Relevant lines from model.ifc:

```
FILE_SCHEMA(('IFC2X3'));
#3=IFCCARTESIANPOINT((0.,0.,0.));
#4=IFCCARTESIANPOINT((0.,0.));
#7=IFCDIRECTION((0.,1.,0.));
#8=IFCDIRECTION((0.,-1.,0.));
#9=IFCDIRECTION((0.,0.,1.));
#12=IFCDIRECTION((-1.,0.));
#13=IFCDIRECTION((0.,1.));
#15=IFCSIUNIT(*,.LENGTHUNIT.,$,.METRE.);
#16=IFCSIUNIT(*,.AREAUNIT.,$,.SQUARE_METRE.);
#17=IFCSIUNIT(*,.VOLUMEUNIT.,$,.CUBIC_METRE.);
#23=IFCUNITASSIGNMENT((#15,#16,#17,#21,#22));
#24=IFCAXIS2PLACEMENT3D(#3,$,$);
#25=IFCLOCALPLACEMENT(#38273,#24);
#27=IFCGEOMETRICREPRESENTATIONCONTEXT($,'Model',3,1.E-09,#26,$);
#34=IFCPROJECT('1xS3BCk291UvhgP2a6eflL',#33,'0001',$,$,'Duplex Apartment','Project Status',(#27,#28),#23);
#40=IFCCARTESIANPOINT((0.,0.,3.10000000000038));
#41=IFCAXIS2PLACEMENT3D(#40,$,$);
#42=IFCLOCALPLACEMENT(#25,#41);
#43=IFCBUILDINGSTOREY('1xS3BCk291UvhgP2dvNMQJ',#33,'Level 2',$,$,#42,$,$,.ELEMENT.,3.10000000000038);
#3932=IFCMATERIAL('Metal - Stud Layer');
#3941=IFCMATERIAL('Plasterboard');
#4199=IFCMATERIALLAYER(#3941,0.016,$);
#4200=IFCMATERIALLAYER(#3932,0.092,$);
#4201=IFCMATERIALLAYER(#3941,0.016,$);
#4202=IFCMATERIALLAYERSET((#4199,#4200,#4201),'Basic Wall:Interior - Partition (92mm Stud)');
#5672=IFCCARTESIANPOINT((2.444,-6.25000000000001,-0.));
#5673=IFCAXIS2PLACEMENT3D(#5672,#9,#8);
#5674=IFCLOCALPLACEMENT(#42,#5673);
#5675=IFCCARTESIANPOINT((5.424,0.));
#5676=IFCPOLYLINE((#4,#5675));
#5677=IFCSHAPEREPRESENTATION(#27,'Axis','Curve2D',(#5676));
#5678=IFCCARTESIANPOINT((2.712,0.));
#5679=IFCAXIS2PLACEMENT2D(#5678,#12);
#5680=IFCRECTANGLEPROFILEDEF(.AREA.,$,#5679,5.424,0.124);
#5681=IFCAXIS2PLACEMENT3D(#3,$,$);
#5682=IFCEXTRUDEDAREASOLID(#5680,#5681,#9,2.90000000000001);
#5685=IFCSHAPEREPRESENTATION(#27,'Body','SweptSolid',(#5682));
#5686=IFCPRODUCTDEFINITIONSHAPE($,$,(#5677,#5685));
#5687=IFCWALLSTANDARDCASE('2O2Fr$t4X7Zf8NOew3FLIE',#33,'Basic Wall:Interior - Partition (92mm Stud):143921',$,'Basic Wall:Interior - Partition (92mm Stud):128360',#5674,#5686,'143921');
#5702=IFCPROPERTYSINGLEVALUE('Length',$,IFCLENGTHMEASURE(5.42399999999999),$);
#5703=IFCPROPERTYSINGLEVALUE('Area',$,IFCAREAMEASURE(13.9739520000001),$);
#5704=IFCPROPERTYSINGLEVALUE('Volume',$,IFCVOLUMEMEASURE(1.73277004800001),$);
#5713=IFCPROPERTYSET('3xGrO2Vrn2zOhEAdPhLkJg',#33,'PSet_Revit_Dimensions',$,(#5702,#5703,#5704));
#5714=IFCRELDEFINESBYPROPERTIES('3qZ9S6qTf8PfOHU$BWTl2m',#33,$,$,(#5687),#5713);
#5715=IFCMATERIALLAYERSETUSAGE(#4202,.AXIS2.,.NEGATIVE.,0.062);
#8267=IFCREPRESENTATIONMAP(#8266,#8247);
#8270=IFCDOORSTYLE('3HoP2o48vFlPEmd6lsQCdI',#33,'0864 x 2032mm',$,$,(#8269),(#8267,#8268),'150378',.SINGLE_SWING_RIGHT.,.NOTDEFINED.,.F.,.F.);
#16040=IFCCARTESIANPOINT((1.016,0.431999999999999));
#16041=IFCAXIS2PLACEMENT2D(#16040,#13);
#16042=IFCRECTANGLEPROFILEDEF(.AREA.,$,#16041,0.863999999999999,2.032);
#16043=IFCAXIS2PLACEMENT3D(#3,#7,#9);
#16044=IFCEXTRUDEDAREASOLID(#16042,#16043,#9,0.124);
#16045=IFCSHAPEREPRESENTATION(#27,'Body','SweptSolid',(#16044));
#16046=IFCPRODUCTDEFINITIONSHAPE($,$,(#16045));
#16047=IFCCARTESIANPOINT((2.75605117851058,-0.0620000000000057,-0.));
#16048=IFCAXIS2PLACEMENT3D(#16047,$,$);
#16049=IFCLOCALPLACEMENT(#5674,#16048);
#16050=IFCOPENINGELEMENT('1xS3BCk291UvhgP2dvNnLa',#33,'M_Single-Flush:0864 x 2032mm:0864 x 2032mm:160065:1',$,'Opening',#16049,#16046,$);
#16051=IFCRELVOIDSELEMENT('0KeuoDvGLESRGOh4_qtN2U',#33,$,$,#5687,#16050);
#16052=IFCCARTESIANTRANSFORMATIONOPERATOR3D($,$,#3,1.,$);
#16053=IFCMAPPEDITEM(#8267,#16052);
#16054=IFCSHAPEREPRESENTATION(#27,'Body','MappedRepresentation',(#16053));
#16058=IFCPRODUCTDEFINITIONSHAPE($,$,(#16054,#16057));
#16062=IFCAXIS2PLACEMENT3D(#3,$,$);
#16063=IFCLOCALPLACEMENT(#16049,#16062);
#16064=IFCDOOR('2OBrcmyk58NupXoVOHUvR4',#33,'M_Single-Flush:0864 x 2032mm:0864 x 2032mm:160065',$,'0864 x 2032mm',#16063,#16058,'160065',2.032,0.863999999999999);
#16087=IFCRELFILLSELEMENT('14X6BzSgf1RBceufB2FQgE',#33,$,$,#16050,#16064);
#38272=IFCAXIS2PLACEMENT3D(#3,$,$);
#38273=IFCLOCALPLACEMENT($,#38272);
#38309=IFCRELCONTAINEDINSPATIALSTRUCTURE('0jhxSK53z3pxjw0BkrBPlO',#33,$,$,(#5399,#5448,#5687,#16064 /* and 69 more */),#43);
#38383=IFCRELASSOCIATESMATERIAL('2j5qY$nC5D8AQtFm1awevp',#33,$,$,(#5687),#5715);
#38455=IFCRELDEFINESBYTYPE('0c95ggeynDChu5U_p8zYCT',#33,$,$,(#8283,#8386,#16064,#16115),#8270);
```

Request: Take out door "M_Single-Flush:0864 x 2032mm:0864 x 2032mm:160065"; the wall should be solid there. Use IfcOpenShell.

```python
import ifcopenshell
import ifcopenshell.api.feature
import ifcopenshell.api.pset
import ifcopenshell.api.root
import ifcopenshell.geom
import ifcopenshell.util.element
import ifcopenshell.util.shape
import ifcopenshell.util.unit

model = ifcopenshell.open("model.ifc")
area_scale = ifcopenshell.util.unit.calculate_unit_scale(model, "AREAUNIT")
volume_scale = ifcopenshell.util.unit.calculate_unit_scale(model, "VOLUMEUNIT")
settings = ifcopenshell.geom.settings()


def volume(element):
    """Net volume in cubic metres, openings subtracted."""
    shape = ifcopenshell.geom.create_shape(settings, element)
    return ifcopenshell.util.shape.get_volume(shape.geometry)


door = model.by_id(16064)
opening = door.FillsVoids[0].RelatingOpeningElement
wall = opening.VoidsElements[0].RelatingBuildingElement
before = volume(wall)

ifcopenshell.api.root.remove_product(model, product=door)
ifcopenshell.api.feature.remove_feature(model, feature=opening)

after = volume(wall)
thickness = 0.124  # wall thickness in metres

# Update the wall's stored quantities.
pset = model.by_id(ifcopenshell.util.element.get_pset(wall, "PSet_Revit_Dimensions", should_inherit=False)["id"])
ifcopenshell.api.pset.edit_pset(model, pset=pset, properties={
    "Area": model.create_entity("IfcAreaMeasure", after / thickness / area_scale),
    "Volume": model.create_entity("IfcVolumeMeasure", after / volume_scale),
})

print(f"wall volume {before:.3f} -> {after:.3f} m3")

model.write("model_updated.ifc")
```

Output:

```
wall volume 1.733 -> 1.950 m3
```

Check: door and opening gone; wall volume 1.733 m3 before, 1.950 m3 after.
